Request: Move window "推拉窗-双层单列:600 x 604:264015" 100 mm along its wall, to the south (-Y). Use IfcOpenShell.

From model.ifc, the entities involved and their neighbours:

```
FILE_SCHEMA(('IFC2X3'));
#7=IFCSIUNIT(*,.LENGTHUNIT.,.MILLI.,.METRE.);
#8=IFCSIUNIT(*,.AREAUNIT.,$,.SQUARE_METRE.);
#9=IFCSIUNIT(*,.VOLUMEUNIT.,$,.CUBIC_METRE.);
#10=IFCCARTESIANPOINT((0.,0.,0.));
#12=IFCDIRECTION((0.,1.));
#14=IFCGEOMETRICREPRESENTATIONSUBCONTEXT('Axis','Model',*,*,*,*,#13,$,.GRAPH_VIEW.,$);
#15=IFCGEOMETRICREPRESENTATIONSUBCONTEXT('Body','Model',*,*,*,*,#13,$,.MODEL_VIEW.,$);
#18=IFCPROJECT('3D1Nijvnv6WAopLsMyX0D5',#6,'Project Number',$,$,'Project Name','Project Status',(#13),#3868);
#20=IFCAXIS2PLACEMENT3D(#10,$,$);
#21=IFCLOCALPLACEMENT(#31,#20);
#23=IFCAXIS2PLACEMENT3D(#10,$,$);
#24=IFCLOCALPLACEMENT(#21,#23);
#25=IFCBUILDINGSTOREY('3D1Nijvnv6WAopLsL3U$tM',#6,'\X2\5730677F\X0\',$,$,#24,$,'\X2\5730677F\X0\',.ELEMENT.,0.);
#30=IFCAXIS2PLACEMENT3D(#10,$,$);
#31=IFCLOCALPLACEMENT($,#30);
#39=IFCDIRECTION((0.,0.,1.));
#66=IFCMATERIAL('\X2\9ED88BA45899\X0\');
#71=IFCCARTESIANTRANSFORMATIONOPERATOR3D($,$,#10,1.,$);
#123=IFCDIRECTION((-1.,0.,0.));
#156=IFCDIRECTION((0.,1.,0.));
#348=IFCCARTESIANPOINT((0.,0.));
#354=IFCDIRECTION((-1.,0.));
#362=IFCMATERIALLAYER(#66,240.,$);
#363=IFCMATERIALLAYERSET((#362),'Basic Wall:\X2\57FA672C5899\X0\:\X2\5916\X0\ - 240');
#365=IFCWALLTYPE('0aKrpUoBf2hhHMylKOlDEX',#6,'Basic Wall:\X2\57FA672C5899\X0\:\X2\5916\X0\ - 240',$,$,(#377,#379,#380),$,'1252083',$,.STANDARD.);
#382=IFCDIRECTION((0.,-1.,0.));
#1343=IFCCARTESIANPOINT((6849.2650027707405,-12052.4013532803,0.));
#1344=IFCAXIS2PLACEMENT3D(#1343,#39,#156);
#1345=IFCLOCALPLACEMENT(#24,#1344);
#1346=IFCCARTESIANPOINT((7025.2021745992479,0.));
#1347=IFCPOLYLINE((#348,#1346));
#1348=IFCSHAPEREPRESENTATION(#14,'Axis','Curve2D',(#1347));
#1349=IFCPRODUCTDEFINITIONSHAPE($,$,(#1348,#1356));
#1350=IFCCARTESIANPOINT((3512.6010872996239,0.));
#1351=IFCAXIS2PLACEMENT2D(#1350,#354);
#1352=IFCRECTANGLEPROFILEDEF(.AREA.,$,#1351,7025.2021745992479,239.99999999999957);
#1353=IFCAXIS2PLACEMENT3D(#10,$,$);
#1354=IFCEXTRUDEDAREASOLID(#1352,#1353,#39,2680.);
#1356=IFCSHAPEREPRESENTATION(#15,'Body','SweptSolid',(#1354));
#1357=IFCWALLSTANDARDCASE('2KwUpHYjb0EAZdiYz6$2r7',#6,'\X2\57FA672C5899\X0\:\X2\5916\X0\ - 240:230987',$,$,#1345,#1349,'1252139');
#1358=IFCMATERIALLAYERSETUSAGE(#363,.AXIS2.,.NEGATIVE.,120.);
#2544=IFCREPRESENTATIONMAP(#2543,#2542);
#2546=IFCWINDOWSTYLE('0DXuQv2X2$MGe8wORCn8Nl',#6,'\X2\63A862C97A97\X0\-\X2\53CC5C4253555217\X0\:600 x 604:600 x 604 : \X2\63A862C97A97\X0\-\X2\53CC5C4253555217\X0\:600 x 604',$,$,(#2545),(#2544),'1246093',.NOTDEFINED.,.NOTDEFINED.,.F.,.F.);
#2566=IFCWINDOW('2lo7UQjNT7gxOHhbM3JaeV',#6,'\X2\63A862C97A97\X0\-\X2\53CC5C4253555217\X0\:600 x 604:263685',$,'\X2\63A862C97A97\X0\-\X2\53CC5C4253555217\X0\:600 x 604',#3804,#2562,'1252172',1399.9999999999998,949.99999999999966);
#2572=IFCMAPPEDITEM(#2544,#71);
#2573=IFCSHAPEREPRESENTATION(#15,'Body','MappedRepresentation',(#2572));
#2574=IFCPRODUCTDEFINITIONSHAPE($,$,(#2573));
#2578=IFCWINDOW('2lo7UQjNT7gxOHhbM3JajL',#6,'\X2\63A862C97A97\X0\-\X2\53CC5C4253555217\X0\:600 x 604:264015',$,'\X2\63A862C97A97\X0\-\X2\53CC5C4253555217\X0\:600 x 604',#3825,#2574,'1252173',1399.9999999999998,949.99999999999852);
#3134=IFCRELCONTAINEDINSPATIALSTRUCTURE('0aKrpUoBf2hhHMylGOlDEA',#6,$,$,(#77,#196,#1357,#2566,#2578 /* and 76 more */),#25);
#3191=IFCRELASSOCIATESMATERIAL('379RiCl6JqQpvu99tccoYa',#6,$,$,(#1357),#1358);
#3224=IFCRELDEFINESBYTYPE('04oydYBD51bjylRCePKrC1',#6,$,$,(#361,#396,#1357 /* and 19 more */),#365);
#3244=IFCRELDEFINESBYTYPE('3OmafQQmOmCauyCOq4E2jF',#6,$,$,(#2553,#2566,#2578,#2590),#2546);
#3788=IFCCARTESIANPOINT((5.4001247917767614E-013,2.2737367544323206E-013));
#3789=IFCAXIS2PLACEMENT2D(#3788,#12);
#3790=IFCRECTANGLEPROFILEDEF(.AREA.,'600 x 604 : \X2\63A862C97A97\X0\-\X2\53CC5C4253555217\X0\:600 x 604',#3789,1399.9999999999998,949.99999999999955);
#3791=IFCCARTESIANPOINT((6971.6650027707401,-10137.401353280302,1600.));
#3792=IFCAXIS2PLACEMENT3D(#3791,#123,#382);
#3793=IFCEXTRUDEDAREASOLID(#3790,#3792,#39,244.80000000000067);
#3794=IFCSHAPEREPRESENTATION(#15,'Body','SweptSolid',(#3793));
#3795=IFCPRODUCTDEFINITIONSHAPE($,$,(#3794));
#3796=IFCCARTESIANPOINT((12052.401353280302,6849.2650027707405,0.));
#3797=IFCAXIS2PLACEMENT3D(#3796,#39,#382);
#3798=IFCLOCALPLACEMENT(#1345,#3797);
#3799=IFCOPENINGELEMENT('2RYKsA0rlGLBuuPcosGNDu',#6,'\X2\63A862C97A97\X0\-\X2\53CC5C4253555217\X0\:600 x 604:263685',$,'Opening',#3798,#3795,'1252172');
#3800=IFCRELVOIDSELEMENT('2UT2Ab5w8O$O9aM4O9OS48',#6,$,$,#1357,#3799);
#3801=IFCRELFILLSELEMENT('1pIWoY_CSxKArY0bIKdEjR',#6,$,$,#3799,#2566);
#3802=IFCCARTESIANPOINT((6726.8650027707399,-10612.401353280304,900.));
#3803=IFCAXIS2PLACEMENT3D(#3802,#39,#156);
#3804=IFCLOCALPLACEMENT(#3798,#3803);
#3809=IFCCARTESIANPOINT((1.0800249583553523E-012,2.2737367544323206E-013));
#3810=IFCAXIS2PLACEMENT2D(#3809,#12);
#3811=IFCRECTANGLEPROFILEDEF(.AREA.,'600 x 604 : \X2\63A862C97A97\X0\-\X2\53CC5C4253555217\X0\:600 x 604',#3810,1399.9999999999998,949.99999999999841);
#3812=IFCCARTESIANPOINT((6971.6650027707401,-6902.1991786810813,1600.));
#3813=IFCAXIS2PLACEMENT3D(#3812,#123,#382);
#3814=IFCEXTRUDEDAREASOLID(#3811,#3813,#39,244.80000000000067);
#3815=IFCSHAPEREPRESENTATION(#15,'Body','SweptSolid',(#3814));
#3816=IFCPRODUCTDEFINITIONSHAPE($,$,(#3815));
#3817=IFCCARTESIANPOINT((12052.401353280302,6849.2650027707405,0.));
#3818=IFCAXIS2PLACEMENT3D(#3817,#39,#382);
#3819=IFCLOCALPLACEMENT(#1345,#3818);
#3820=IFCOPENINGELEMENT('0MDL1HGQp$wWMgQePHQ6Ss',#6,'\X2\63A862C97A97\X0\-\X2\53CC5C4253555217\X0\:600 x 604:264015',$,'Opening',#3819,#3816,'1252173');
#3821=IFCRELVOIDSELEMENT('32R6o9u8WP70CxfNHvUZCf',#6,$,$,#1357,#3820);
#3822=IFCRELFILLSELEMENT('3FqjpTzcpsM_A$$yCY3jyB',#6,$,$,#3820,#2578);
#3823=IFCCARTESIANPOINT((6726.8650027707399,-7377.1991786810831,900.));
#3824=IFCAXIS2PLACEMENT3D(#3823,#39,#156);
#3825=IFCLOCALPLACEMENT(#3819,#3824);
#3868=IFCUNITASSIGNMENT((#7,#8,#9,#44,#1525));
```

```python
import ifcopenshell
import ifcopenshell.api.geometry
import ifcopenshell.util.placement

model = ifcopenshell.open("model.ifc")

window = model.by_id(2578)
opening = window.FillsVoids[0].RelatingOpeningElement
wall = opening.VoidsElements[0].RelatingBuildingElement

wall_matrix = ifcopenshell.util.placement.get_local_placement(wall.ObjectPlacement)
shift = wall_matrix[:3, 0] * -100.0
before = ifcopenshell.util.placement.get_local_placement(window.ObjectPlacement)[:3, 3].copy()

# The window is placed relative to its opening, so it follows when the opening moves.
matrix = ifcopenshell.util.placement.get_local_placement(opening.ObjectPlacement)
matrix[:3, 3] += shift
ifcopenshell.api.geometry.edit_object_placement(
    model, product=opening, matrix=matrix, is_si=False, should_transform_children=True
)

after = ifcopenshell.util.placement.get_local_placement(window.ObjectPlacement)[:3, 3]
print("window moved by", (after - before).round(3) + 0.0)

model.write("model_edited.ifc")
```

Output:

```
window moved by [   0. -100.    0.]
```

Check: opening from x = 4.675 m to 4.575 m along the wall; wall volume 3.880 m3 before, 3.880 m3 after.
